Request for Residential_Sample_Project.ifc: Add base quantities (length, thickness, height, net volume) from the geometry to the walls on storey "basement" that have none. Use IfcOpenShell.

First a look at what the model holds.

```python
import ifcopenshell
import ifcopenshell.util.element
import ifcopenshell.util.unit

model = ifcopenshell.open("Residential_Sample_Project.ifc")
print(model.schema)
for unit_type in ("LENGTHUNIT", "AREAUNIT", "VOLUMEUNIT"):
    print(unit_type, ifcopenshell.util.unit.calculate_unit_scale(model, unit_type))
storey = next(s for s in model.by_type("IfcBuildingStorey") if s.Name == "basement")
walls = [e for e in ifcopenshell.util.element.get_decomposition(storey) if e.is_a("IfcWall")]
for e in sorted(walls, key=lambda e: e.id()):
    print(e.id(), e.is_a(), e.Name, list(ifcopenshell.util.element.get_psets(e, qtos_only=True)), sep=" | ")
```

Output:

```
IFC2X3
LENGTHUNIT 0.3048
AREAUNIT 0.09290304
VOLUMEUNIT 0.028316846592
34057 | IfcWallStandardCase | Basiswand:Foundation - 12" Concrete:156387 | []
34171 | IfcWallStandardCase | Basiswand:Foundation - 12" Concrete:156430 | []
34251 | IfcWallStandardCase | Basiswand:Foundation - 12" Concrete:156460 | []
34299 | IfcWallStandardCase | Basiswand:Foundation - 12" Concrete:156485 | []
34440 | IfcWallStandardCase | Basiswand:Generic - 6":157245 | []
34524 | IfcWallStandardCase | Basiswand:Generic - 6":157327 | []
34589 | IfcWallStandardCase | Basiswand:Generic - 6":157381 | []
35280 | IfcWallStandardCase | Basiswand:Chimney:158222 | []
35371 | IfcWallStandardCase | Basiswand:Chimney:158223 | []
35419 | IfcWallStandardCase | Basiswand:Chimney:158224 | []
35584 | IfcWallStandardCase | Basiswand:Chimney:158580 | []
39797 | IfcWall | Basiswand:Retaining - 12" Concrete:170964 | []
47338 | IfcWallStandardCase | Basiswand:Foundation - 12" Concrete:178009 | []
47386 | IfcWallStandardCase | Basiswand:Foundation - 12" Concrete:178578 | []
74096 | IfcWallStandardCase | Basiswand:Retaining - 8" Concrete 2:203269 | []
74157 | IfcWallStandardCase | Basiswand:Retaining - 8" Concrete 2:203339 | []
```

```python
import ifcopenshell
import ifcopenshell.api.pset
import ifcopenshell.geom
import ifcopenshell.util.element
import ifcopenshell.util.shape
import ifcopenshell.util.unit

model = ifcopenshell.open("Residential_Sample_Project.ifc")
unit_scale = ifcopenshell.util.unit.calculate_unit_scale(model)
volume_scale = ifcopenshell.util.unit.calculate_unit_scale(model, "VOLUMEUNIT")
settings = ifcopenshell.geom.settings()

storey = next(s for s in model.by_type("IfcBuildingStorey") if s.Name == "basement")
walls = [e for e in ifcopenshell.util.element.get_decomposition(storey) if e.is_a("IfcWall")]

for e in sorted(walls, key=lambda e: e.id()):
    if ifcopenshell.util.element.get_psets(e, qtos_only=True, should_inherit=False):
        continue
    # Geometry comes back in metres, in the element's own axes.
    shape = ifcopenshell.geom.create_shape(settings, e)
    values = {
        "Length": ifcopenshell.util.shape.get_x(shape.geometry) / unit_scale,
        "Width": ifcopenshell.util.shape.get_y(shape.geometry) / unit_scale,
        "Height": ifcopenshell.util.shape.get_z(shape.geometry) / unit_scale,
        "NetVolume": ifcopenshell.util.shape.get_volume(shape.geometry) / volume_scale,
    }
    qto = ifcopenshell.api.pset.add_qto(model, product=e, name="BaseQuantities")
    ifcopenshell.api.pset.edit_qto(model, qto=qto, properties=values)
    print(e.id(), {k: round(v, 3) for k, v in values.items()})

model.write("Residential_Sample_Project-out.ifc")
```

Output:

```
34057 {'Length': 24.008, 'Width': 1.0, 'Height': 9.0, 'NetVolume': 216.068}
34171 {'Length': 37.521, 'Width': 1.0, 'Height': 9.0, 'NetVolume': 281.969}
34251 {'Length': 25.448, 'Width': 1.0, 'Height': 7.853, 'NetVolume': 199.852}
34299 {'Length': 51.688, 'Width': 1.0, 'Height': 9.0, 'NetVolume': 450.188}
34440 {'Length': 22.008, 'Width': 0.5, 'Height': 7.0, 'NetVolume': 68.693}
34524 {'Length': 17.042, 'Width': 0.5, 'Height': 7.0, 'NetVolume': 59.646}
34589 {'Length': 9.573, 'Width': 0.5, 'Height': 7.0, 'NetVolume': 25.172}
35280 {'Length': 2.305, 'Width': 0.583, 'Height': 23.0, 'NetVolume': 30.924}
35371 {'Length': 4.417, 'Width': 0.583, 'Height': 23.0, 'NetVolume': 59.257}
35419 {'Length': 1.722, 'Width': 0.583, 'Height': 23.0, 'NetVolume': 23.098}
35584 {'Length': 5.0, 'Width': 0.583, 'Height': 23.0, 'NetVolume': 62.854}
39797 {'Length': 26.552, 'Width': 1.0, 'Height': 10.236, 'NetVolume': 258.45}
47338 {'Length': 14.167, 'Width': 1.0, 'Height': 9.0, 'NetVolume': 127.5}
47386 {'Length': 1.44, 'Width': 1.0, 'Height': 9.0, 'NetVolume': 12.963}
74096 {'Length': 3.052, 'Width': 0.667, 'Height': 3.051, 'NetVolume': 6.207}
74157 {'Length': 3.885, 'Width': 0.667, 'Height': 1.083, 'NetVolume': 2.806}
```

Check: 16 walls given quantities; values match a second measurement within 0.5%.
